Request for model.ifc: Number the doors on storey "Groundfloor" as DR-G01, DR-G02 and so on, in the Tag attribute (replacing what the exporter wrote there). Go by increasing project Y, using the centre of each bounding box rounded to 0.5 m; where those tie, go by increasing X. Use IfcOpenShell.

First a look at what the model holds.

```python
import ifcopenshell
import ifcopenshell.util.element
import ifcopenshell.util.placement

model = ifcopenshell.open("model.ifc")
print(model.schema)
storey = next(s for s in model.by_type("IfcBuildingStorey") if s.Name == "Groundfloor")
doors = [e for e in ifcopenshell.util.element.get_decomposition(storey) if e.is_a("IfcDoor")]
for e in sorted(doors, key=lambda e: e.id()):
    origin = ifcopenshell.util.placement.get_local_placement(e.ObjectPlacement)[:3, 3]
    print(e.id(), e.Tag, e.Name, origin.round(2) + 0.0, sep=" | ")
```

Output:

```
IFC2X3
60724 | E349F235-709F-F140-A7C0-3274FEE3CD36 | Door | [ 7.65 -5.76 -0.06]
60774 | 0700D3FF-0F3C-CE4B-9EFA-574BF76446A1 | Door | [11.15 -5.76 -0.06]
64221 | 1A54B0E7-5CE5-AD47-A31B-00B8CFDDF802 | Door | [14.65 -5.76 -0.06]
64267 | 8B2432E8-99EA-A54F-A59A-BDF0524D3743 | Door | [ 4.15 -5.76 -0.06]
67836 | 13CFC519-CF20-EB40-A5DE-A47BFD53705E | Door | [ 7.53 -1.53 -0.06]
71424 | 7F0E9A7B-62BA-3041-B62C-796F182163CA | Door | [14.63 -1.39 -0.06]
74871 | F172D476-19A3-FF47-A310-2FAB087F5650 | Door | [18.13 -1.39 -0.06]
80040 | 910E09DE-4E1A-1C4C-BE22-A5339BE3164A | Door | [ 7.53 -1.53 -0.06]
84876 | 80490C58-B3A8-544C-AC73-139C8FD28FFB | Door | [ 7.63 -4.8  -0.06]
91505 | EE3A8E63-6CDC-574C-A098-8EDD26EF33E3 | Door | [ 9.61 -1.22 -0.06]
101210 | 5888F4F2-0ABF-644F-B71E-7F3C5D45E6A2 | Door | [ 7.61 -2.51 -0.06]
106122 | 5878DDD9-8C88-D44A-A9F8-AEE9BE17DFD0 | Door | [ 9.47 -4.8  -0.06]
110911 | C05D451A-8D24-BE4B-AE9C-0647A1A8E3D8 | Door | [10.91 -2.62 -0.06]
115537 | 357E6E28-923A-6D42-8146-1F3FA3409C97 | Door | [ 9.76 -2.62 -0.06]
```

```python
import ifcopenshell
import ifcopenshell.geom
import ifcopenshell.util.element
import ifcopenshell.util.shape

model = ifcopenshell.open("model.ifc")
settings = ifcopenshell.geom.settings()
settings.set("use-world-coords", True)


def centre(element):
    shape = ifcopenshell.geom.create_shape(settings, element)
    return ifcopenshell.util.shape.get_bbox_centroid(shape.geometry)


storey = next(s for s in model.by_type("IfcBuildingStorey") if s.Name == "Groundfloor")
doors = [e for e in ifcopenshell.util.element.get_decomposition(storey) if e.is_a("IfcDoor")]

# Insertion points can sit at a corner or the storey origin, so sort by the geometry (in metres).
centres = {e: centre(e) for e in doors}
doors.sort(key=lambda e: (round(centres[e][1] / 0.5), centres[e][0]))

for i, e in enumerate(doors, start=1):
    number = f"DR-G{i:02d}"
    e.Tag = number
    print(e.id(), number)

model.write("model_rev.ifc")
```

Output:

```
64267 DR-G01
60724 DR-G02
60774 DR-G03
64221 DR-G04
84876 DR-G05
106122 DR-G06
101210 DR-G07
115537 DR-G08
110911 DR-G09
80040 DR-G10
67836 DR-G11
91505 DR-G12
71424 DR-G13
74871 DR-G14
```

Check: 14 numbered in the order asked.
